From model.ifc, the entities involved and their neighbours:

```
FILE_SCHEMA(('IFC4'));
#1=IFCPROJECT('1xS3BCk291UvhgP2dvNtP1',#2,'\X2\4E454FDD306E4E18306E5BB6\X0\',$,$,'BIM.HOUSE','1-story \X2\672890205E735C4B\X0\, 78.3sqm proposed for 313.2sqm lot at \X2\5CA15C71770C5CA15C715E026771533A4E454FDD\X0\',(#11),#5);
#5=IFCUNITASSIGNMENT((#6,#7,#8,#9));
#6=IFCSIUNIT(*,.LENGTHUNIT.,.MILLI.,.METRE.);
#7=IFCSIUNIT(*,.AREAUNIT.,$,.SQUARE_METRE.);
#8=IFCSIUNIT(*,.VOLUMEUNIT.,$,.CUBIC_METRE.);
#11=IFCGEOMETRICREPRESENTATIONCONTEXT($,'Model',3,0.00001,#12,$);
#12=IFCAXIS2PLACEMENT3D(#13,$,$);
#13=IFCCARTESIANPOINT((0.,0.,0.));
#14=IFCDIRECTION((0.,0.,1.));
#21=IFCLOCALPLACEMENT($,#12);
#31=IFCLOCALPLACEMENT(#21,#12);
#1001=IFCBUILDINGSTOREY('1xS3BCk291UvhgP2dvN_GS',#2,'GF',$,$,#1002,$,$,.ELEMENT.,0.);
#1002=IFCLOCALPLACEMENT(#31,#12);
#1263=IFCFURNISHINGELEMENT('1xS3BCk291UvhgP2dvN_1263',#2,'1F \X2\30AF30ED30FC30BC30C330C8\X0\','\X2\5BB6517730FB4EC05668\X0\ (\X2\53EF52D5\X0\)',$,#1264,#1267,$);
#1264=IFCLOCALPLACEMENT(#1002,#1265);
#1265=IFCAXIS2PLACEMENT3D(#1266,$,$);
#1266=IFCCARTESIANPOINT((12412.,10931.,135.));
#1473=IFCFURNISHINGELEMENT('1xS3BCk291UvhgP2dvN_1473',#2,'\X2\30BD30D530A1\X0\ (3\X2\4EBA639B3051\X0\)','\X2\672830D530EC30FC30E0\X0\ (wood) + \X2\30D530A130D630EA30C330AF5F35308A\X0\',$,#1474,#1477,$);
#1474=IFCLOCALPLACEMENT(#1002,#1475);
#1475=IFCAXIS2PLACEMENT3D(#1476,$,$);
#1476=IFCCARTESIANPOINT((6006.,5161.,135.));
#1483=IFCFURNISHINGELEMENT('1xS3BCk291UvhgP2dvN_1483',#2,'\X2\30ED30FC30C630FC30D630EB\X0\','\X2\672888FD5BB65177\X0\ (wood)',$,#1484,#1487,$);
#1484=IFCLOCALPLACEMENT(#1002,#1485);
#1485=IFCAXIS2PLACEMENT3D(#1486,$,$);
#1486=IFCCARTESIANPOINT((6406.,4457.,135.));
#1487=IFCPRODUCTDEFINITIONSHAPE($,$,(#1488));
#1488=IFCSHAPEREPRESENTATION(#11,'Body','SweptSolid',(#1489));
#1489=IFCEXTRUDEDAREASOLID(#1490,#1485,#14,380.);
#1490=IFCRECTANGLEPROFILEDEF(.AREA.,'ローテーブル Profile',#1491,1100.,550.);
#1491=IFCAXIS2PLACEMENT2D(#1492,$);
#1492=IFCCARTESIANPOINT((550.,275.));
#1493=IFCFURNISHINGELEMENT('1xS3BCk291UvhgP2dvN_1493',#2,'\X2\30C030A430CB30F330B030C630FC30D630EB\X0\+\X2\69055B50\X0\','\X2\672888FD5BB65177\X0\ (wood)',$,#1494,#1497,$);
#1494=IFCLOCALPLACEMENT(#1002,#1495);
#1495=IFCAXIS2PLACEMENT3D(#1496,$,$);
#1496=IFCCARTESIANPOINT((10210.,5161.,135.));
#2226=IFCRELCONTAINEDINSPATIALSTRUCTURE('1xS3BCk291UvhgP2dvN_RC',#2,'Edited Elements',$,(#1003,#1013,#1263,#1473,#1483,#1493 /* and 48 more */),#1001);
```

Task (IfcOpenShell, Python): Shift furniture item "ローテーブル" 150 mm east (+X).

```python
import ifcopenshell
import ifcopenshell.api.geometry
import ifcopenshell.util.placement

model = ifcopenshell.open("model.ifc")

item = model.by_guid("1xS3BCk291UvhgP2dvN_1483")
matrix = ifcopenshell.util.placement.get_local_placement(item.ObjectPlacement)
matrix[0, 3] += 150.0
ifcopenshell.api.geometry.edit_object_placement(model, product=item, matrix=matrix, is_si=False)

print(ifcopenshell.util.placement.get_local_placement(item.ObjectPlacement).round(3) + 0.0)

model.write("model-out.ifc")
```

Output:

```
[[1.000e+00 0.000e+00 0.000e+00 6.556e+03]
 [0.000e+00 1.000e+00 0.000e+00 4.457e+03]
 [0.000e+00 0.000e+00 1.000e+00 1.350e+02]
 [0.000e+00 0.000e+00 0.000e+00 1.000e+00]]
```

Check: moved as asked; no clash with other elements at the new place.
